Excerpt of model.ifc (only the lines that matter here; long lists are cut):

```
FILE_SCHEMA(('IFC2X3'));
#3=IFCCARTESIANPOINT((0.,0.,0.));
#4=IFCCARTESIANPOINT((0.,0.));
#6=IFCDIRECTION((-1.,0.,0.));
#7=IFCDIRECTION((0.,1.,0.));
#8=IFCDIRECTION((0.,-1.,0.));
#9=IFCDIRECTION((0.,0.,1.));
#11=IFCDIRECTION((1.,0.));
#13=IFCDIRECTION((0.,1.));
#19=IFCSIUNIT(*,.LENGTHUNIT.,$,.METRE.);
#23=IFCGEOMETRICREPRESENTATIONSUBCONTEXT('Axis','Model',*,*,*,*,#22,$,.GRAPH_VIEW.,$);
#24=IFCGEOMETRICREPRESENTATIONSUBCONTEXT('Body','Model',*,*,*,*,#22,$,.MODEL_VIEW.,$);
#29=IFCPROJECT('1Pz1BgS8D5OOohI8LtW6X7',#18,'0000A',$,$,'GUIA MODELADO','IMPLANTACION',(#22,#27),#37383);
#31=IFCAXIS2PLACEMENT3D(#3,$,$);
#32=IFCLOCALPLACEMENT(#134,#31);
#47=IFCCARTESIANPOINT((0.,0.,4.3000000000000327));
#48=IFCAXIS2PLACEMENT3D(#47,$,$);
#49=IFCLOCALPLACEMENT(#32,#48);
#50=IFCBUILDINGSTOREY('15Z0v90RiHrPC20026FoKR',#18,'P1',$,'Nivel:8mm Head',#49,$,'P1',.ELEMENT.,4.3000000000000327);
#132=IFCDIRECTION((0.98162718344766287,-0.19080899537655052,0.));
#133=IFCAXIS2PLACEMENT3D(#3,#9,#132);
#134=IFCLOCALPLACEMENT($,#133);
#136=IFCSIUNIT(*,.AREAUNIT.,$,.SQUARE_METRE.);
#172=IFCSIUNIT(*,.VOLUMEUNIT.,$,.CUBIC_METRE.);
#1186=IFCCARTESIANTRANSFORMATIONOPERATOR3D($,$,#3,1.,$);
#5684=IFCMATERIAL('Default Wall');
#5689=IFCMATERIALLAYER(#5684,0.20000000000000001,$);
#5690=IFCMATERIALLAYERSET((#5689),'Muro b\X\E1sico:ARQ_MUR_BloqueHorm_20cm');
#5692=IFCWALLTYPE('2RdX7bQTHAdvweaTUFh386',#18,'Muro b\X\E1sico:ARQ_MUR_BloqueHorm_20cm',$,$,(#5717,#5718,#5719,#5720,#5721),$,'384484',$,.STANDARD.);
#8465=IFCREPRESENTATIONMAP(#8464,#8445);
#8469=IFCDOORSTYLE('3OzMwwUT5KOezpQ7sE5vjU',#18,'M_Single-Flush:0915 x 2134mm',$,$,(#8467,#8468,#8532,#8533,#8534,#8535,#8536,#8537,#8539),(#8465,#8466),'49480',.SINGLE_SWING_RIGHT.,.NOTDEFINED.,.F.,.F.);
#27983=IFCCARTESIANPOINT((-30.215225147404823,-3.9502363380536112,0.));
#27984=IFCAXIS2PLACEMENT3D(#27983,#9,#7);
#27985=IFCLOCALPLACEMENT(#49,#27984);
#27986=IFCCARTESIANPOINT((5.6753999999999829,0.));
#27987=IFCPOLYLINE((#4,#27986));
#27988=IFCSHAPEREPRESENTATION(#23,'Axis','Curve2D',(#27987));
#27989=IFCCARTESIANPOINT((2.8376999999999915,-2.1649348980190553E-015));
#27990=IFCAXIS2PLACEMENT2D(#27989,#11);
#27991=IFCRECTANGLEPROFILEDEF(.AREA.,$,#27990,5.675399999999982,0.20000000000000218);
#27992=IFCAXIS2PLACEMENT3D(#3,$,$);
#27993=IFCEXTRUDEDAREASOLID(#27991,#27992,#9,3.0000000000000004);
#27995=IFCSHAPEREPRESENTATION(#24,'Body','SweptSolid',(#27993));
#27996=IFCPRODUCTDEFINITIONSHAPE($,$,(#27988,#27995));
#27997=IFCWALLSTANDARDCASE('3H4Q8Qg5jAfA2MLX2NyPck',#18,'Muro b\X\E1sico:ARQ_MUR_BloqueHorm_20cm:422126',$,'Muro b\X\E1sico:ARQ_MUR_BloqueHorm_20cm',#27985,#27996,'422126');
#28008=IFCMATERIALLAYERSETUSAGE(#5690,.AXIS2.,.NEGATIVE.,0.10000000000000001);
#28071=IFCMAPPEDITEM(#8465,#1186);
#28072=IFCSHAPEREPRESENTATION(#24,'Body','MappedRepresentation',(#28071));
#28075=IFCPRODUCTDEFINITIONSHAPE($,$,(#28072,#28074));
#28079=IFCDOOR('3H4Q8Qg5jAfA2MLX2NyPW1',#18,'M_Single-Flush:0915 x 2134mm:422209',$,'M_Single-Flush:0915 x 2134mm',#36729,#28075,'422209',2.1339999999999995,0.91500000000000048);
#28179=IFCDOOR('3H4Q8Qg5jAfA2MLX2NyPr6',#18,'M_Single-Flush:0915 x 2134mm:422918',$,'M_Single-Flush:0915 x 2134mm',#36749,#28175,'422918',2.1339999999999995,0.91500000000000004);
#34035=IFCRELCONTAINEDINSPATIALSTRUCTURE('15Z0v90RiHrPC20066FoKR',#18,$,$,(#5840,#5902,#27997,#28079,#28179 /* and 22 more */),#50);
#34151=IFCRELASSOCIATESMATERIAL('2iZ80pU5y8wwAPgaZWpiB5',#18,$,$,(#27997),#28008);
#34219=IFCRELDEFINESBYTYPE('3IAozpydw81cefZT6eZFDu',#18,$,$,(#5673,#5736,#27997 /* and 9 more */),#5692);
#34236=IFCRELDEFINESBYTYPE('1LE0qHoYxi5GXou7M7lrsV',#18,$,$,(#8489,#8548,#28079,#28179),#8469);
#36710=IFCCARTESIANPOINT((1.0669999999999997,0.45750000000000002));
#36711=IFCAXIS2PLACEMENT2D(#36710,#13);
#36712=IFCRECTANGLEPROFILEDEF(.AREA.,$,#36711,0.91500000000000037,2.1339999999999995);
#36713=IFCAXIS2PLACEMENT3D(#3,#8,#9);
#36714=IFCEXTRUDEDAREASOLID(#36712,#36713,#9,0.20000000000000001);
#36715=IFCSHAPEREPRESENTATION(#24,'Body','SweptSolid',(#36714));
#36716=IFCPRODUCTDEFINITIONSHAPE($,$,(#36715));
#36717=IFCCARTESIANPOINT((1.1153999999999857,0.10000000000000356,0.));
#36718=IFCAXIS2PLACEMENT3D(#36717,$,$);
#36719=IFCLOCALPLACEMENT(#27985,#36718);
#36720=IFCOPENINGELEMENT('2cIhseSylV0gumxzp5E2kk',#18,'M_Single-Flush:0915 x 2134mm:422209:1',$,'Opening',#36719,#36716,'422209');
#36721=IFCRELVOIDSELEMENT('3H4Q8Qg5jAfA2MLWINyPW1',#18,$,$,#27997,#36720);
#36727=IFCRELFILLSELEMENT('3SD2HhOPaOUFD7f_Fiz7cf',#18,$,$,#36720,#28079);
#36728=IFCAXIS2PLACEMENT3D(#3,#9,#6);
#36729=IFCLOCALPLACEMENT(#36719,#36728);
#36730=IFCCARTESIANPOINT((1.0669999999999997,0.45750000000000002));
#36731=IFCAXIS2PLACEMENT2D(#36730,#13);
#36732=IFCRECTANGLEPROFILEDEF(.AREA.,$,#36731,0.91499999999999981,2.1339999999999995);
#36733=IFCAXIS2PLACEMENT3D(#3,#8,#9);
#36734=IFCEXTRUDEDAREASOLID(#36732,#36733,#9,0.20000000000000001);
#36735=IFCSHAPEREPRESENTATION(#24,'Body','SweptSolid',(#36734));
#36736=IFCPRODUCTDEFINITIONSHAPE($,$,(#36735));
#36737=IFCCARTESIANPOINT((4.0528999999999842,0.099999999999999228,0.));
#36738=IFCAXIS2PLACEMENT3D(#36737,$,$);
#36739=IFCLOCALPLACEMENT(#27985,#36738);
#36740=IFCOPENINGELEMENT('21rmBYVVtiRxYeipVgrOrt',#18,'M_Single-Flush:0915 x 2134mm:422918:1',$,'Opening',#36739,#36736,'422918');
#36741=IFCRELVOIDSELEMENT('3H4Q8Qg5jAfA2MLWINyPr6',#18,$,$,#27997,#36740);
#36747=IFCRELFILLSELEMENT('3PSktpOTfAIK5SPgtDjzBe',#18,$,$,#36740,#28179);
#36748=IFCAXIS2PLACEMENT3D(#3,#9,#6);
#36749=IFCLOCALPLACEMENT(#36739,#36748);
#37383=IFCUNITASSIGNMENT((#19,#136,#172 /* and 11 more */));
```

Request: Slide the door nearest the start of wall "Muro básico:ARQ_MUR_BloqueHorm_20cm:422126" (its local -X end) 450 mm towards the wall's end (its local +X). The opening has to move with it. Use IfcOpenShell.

```python
import ifcopenshell
import ifcopenshell.api.geometry
import ifcopenshell.util.placement
import ifcopenshell.util.unit

model = ifcopenshell.open("model.ifc")
unit_scale = ifcopenshell.util.unit.calculate_unit_scale(model)

door = model.by_guid("3H4Q8Qg5jAfA2MLX2NyPW1")
opening = door.FillsVoids[0].RelatingOpeningElement
wall = opening.VoidsElements[0].RelatingBuildingElement

wall_matrix = ifcopenshell.util.placement.get_local_placement(wall.ObjectPlacement)
shift = wall_matrix[:3, 0] * 0.45 / unit_scale
before = ifcopenshell.util.placement.get_local_placement(door.ObjectPlacement)[:3, 3].copy()

# The door is placed relative to its opening, so it follows when the opening moves.
matrix = ifcopenshell.util.placement.get_local_placement(opening.ObjectPlacement)
matrix[:3, 3] += shift
ifcopenshell.api.geometry.edit_object_placement(
    model, product=opening, matrix=matrix, is_si=False, should_transform_children=True
)

after = ifcopenshell.util.placement.get_local_placement(door.ObjectPlacement)[:3, 3]
print("door moved by", (after - before).round(3) + 0.0)

model.write("model-out.ifc")
```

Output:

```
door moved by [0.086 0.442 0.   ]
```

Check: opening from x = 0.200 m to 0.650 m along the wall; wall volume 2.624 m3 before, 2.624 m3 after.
